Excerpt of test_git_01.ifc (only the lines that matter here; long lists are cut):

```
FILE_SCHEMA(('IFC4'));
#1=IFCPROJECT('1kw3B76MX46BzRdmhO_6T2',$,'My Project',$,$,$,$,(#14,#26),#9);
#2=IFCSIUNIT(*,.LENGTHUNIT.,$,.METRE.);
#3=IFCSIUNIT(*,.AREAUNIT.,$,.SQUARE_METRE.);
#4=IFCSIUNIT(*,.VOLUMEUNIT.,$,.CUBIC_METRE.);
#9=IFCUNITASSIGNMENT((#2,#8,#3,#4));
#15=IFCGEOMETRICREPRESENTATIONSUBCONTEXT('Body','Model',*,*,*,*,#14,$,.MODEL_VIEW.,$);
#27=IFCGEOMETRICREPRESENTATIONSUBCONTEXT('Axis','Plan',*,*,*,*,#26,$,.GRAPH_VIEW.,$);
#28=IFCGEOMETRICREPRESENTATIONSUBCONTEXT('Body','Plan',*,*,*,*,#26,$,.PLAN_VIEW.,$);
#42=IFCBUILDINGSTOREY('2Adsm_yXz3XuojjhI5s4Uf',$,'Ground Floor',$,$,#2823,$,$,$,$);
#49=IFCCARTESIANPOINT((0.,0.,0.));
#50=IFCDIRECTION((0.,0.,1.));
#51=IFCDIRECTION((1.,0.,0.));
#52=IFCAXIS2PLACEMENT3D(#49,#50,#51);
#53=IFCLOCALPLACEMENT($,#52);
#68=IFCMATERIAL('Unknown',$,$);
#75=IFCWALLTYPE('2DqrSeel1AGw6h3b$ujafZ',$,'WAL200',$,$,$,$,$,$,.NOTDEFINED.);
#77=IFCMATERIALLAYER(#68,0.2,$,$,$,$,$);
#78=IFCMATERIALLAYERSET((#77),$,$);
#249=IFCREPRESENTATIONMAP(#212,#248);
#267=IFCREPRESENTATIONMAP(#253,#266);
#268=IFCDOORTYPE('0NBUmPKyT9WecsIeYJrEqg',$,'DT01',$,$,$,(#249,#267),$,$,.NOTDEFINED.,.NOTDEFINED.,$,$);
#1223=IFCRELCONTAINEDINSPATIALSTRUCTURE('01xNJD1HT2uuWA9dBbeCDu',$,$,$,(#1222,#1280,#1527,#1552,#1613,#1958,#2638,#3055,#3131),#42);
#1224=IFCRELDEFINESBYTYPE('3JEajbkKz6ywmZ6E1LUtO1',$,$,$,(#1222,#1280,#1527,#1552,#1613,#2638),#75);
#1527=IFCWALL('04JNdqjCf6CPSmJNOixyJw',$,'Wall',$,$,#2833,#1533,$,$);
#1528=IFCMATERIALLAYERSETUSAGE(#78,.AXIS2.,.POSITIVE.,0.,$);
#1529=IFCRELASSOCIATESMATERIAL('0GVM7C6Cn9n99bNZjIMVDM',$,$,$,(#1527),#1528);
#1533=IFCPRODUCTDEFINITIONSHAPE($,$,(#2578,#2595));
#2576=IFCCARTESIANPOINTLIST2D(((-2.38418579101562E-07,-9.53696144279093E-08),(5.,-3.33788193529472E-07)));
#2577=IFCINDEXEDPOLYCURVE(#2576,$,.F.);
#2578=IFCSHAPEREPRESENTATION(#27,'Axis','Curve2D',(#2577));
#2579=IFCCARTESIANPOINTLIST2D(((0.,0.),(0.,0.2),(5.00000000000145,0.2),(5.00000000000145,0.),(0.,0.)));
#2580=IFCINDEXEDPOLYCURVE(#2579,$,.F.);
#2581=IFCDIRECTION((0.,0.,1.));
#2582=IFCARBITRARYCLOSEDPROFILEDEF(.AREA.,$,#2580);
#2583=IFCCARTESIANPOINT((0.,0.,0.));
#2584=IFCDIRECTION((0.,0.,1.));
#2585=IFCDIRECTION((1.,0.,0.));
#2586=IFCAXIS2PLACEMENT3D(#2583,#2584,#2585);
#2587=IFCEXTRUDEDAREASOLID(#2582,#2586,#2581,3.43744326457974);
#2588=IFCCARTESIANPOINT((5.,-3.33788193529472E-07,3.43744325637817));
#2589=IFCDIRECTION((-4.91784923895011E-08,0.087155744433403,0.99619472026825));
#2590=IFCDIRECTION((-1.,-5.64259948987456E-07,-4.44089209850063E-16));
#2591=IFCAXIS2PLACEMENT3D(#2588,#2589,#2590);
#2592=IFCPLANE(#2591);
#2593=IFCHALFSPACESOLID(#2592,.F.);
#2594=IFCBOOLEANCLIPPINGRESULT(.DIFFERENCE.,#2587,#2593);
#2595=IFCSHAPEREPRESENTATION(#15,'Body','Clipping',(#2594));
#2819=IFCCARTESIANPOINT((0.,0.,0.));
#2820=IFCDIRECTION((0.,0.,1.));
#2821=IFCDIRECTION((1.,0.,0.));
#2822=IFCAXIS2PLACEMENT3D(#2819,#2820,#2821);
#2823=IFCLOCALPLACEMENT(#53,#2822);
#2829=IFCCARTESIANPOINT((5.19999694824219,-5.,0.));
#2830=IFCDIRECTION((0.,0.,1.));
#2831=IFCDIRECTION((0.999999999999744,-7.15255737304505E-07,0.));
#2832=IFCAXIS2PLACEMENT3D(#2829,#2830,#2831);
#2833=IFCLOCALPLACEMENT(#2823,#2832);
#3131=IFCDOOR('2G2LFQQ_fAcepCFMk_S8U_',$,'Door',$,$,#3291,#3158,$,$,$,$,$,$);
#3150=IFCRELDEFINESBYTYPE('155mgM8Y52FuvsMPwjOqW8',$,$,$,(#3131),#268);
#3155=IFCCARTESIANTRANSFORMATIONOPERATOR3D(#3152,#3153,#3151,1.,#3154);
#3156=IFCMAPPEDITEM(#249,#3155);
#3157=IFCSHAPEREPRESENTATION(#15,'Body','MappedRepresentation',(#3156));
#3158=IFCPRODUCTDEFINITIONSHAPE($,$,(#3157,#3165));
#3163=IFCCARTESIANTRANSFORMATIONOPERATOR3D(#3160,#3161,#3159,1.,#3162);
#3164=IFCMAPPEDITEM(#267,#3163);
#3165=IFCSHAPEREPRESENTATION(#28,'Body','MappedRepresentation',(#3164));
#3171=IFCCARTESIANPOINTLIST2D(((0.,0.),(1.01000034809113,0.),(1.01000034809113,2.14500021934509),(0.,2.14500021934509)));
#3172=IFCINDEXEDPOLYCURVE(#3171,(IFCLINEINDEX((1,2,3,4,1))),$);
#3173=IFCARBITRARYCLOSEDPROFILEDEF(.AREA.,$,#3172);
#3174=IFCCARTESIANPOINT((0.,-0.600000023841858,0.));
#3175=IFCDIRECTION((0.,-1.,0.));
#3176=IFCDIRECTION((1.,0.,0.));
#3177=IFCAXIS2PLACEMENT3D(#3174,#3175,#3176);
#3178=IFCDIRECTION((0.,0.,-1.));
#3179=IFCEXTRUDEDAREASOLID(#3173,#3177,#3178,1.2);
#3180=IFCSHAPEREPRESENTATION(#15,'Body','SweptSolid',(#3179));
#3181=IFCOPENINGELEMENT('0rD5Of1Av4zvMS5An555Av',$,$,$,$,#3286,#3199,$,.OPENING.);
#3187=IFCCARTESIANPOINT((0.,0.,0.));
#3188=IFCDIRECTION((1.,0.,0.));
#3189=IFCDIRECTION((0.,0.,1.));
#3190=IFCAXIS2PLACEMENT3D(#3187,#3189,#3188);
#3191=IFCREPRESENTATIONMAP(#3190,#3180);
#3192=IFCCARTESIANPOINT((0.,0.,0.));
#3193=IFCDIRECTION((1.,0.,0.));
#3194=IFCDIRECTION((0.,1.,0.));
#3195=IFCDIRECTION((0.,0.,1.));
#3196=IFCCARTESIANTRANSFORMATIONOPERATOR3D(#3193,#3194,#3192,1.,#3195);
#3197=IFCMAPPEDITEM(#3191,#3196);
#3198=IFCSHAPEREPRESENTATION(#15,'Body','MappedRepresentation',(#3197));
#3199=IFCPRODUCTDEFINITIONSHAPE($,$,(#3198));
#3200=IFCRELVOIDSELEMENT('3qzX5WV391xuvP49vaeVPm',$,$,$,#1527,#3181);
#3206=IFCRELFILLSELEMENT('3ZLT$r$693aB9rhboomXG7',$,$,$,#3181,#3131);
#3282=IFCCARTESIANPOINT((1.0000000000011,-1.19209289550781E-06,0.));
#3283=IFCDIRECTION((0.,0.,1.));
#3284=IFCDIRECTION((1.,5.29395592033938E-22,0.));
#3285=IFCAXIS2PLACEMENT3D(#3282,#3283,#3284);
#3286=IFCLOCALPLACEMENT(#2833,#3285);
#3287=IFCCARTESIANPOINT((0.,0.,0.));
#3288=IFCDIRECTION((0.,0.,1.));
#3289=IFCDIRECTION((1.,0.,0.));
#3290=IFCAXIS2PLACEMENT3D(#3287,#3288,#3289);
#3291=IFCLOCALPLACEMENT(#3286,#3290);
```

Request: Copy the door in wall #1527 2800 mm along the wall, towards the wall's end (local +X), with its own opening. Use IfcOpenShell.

```python
import ifcopenshell
import ifcopenshell.api.feature
import ifcopenshell.api.geometry
import ifcopenshell.api.root
import ifcopenshell.geom
import ifcopenshell.util.element
import ifcopenshell.util.placement
import ifcopenshell.util.shape

model = ifcopenshell.open("test_git_01.ifc")
settings = ifcopenshell.geom.settings()


def volume(element):
    """Net volume in cubic metres, openings subtracted."""
    shape = ifcopenshell.geom.create_shape(settings, element)
    return ifcopenshell.util.shape.get_volume(shape.geometry)


door = model.by_guid("2G2LFQQ_fAcepCFMk_S8U_")
opening = door.FillsVoids[0].RelatingOpeningElement
wall = opening.VoidsElements[0].RelatingBuildingElement
before = volume(wall)
shift = ifcopenshell.util.placement.get_local_placement(wall.ObjectPlacement)[:3, 0] * 2.8

# copy_class copies the void relationship, type, container and properties, but no geometry.
new_opening = ifcopenshell.api.root.copy_class(model, product=opening)
new_opening.Representation = ifcopenshell.util.element.copy_deep(
    model, opening.Representation, exclude=["IfcGeometricRepresentationContext", "IfcRepresentationMap"]
)
new_door = ifcopenshell.api.root.copy_class(model, product=door)
new_door.Representation = ifcopenshell.util.element.copy_deep(
    model, door.Representation, exclude=["IfcGeometricRepresentationContext", "IfcRepresentationMap"]
)
ifcopenshell.api.feature.add_filling(model, opening=new_opening, element=new_door)

for old, new in ((opening, new_opening), (door, new_door)):
    matrix = ifcopenshell.util.placement.get_local_placement(old.ObjectPlacement)
    matrix[:3, 3] += shift
    ifcopenshell.api.geometry.edit_object_placement(model, product=new, matrix=matrix, is_si=False)

after = volume(wall)

print(f"wall volume {before:.3f} -> {after:.3f} m3")

model.write("test_git_01_updated.ifc")
```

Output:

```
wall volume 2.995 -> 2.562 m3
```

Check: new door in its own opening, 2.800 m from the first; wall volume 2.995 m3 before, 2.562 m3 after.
